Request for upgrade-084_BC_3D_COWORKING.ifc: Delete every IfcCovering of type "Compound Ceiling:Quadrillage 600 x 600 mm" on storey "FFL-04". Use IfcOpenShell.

First a look at what the model holds.

```python
import ifcopenshell
import ifcopenshell.util.element

model = ifcopenshell.open("upgrade-084_BC_3D_COWORKING.ifc")
print(model.schema)
storey = next(s for s in model.by_type("IfcBuildingStorey") if s.Name == "FFL-04")
coverings = [e for e in ifcopenshell.util.element.get_decomposition(storey) if e.is_a("IfcCovering")]
seen = {}
for e in coverings:
    element_type = ifcopenshell.util.element.get_type(e)
    name = element_type.Name if element_type not in (None, e) else None
    seen[name] = seen.get(name, 0) + 1
for name, count in sorted(seen.items(), key=str):
    print(count, "x", name)
```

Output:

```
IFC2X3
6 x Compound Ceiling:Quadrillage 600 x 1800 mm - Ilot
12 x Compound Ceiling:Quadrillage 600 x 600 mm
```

```python
import ifcopenshell
import ifcopenshell.api.root
import ifcopenshell.util.element

model = ifcopenshell.open("upgrade-084_BC_3D_COWORKING.ifc")

storey = next(s for s in model.by_type("IfcBuildingStorey") if s.Name == "FFL-04")
coverings = [e for e in ifcopenshell.util.element.get_decomposition(storey) if e.is_a("IfcCovering")]
targets = [e for e in coverings if (t := ifcopenshell.util.element.get_type(e)) not in (None, e) and t.Name == "Compound Ceiling:Quadrillage 600 x 600 mm"]

for e in targets:
    ifcopenshell.api.root.remove_product(model, product=e)
print(len(targets), "removed")

model.write("upgrade-084_BC_3D_COWORKING_updated.ifc")
```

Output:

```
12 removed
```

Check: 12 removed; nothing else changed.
